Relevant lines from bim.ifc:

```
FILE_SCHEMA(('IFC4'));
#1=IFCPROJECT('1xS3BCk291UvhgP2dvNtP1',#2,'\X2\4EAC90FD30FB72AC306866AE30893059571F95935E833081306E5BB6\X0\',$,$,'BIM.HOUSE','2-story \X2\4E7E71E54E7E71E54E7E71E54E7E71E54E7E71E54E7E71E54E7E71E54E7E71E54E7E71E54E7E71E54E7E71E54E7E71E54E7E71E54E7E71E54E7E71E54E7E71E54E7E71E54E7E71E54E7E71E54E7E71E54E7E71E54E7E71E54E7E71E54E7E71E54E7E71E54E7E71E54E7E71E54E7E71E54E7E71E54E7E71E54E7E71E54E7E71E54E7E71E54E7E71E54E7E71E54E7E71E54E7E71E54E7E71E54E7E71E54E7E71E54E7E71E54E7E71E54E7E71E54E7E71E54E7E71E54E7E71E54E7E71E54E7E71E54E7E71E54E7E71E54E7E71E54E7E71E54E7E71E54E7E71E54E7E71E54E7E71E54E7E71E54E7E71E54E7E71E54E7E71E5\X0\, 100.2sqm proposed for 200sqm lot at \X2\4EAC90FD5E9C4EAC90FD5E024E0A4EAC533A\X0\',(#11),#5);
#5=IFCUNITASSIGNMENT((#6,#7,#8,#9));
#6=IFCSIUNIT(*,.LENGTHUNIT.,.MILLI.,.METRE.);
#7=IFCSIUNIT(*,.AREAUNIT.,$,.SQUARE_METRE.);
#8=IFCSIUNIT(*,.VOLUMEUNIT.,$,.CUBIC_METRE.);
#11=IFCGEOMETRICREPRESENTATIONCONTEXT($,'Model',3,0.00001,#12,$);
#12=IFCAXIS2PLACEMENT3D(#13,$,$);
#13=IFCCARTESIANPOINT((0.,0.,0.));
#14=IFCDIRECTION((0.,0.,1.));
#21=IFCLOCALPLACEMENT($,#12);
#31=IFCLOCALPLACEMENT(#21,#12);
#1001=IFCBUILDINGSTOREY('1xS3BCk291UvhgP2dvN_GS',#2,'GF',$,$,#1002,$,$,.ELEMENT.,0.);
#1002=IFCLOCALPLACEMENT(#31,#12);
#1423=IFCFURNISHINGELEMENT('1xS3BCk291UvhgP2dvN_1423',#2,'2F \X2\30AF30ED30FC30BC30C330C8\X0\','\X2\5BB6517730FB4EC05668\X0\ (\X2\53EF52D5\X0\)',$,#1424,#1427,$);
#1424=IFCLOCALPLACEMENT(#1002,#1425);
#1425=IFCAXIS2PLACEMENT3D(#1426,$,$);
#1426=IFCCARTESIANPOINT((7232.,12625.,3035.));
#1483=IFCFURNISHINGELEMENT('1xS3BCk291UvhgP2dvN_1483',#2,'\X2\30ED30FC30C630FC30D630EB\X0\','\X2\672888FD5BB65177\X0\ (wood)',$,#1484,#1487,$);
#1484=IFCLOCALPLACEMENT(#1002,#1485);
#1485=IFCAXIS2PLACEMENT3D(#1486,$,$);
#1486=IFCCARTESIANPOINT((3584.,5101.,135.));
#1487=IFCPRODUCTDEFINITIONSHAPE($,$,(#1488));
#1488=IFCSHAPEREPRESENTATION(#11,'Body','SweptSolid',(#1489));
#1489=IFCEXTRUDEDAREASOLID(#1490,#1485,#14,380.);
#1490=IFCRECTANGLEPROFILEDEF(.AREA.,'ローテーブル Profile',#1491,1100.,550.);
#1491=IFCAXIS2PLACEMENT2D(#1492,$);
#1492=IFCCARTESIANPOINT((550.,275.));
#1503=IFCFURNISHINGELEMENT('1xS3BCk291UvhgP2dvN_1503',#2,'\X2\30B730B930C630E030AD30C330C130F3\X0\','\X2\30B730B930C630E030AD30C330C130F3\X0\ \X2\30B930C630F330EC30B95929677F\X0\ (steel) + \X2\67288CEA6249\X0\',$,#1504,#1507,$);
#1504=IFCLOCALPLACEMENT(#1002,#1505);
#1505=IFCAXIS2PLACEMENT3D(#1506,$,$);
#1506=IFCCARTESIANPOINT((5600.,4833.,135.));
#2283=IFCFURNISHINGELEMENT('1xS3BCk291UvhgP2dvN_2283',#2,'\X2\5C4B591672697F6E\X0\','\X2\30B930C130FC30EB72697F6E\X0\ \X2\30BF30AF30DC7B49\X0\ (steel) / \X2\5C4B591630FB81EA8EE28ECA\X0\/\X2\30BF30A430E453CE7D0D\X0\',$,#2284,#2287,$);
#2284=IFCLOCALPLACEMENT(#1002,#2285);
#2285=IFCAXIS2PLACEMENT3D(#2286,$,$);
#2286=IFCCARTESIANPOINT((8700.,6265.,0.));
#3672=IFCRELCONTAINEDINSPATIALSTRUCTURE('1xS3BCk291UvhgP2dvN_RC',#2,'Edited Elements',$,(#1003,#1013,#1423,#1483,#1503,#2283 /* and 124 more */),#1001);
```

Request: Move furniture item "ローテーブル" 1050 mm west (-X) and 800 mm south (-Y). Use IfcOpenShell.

```python
import ifcopenshell
import ifcopenshell.api.geometry
import ifcopenshell.util.placement

model = ifcopenshell.open("bim.ifc")

item = model.by_guid("1xS3BCk291UvhgP2dvN_1483")
matrix = ifcopenshell.util.placement.get_local_placement(item.ObjectPlacement)
matrix[0, 3] -= 1050.0
matrix[1, 3] -= 800.0
ifcopenshell.api.geometry.edit_object_placement(model, product=item, matrix=matrix, is_si=False)

print(ifcopenshell.util.placement.get_local_placement(item.ObjectPlacement).round(3) + 0.0)

model.write("bim_rev.ifc")
```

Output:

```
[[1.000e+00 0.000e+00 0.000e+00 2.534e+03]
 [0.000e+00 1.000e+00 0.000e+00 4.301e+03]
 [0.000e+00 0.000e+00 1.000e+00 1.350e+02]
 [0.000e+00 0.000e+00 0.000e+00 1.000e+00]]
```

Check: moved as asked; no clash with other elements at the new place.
